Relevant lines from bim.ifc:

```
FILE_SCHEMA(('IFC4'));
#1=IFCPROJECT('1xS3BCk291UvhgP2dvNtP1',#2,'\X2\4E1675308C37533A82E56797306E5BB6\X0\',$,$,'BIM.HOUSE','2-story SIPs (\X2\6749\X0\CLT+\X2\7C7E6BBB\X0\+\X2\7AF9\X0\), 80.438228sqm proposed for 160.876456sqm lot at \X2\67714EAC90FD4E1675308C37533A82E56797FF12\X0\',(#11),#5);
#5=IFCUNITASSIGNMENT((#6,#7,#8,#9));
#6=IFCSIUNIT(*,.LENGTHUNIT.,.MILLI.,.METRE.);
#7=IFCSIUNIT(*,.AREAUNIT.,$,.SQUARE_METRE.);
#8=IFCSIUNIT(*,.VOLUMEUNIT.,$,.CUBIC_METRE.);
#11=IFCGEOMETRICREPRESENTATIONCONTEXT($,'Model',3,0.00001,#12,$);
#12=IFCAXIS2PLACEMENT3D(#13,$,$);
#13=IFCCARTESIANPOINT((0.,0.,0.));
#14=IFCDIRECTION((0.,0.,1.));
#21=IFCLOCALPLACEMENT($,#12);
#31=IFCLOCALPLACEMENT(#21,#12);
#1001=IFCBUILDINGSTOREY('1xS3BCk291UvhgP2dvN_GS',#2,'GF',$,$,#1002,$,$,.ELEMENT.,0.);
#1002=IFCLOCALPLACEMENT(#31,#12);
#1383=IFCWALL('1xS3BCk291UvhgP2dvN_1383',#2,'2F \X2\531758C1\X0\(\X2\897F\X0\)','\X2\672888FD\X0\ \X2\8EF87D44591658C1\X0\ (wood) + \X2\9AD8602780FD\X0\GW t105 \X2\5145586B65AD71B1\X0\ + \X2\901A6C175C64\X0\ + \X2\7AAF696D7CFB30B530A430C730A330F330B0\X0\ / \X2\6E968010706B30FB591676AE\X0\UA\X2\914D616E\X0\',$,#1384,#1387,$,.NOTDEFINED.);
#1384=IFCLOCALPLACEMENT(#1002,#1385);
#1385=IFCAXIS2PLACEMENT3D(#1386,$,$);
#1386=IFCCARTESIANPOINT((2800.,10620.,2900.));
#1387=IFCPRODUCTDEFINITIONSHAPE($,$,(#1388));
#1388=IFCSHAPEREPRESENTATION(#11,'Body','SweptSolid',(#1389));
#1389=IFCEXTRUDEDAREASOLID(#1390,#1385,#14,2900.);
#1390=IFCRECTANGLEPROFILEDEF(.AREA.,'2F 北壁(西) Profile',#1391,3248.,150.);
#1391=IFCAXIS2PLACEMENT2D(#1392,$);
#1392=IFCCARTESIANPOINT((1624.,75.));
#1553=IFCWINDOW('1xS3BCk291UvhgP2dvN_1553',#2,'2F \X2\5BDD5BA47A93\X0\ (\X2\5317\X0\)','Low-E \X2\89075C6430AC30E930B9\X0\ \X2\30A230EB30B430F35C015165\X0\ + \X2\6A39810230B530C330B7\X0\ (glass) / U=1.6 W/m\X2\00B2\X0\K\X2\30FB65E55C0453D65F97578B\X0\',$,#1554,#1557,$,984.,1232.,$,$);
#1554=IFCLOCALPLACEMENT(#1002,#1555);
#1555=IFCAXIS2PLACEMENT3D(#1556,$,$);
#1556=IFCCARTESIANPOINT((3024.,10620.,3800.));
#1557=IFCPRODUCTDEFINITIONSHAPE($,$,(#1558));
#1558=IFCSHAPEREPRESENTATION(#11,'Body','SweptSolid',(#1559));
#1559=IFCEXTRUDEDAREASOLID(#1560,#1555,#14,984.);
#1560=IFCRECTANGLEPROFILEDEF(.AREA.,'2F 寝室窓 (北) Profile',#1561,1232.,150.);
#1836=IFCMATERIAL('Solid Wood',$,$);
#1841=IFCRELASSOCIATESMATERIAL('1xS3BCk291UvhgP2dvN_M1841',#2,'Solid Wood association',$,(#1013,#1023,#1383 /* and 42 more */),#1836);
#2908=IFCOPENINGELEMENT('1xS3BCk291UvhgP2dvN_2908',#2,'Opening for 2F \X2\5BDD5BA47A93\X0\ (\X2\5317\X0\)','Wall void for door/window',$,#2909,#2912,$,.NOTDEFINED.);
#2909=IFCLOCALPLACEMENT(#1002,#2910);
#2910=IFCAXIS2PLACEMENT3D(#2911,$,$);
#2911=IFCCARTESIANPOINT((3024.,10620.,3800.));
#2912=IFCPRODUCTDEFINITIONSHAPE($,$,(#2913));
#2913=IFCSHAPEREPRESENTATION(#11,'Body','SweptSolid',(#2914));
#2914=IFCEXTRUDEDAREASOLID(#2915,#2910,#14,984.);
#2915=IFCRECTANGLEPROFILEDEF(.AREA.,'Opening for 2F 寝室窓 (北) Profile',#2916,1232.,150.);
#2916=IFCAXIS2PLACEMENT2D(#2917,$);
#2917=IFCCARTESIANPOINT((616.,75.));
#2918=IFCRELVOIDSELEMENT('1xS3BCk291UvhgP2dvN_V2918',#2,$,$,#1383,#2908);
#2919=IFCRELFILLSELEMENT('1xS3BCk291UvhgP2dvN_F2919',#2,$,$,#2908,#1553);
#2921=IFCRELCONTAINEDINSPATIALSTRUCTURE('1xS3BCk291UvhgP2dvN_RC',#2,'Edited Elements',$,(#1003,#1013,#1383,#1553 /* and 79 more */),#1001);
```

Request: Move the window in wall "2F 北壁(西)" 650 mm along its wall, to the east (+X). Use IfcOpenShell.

```python
import ifcopenshell
import ifcopenshell.api.geometry
import ifcopenshell.util.placement
import ifcopenshell.util.unit

model = ifcopenshell.open("bim.ifc")
unit_scale = ifcopenshell.util.unit.calculate_unit_scale(model)

window = model.by_guid("1xS3BCk291UvhgP2dvN_1553")
opening = window.FillsVoids[0].RelatingOpeningElement
wall = opening.VoidsElements[0].RelatingBuildingElement

wall_matrix = ifcopenshell.util.placement.get_local_placement(wall.ObjectPlacement)
shift = wall_matrix[:3, 0] * 0.65 / unit_scale
before = ifcopenshell.util.placement.get_local_placement(window.ObjectPlacement)[:3, 3].copy()

# The window is not placed relative to its opening, so move both.
for product in (opening, window):
    matrix = ifcopenshell.util.placement.get_local_placement(product.ObjectPlacement)
    matrix[:3, 3] += shift
    ifcopenshell.api.geometry.edit_object_placement(model, product=product, matrix=matrix, is_si=False)

after = ifcopenshell.util.placement.get_local_placement(window.ObjectPlacement)[:3, 3]
print("window moved by", (after - before).round(3) + 0.0)

model.write("bim_edited.ifc")
```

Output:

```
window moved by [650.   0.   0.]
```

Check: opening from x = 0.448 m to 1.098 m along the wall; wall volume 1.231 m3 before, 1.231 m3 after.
